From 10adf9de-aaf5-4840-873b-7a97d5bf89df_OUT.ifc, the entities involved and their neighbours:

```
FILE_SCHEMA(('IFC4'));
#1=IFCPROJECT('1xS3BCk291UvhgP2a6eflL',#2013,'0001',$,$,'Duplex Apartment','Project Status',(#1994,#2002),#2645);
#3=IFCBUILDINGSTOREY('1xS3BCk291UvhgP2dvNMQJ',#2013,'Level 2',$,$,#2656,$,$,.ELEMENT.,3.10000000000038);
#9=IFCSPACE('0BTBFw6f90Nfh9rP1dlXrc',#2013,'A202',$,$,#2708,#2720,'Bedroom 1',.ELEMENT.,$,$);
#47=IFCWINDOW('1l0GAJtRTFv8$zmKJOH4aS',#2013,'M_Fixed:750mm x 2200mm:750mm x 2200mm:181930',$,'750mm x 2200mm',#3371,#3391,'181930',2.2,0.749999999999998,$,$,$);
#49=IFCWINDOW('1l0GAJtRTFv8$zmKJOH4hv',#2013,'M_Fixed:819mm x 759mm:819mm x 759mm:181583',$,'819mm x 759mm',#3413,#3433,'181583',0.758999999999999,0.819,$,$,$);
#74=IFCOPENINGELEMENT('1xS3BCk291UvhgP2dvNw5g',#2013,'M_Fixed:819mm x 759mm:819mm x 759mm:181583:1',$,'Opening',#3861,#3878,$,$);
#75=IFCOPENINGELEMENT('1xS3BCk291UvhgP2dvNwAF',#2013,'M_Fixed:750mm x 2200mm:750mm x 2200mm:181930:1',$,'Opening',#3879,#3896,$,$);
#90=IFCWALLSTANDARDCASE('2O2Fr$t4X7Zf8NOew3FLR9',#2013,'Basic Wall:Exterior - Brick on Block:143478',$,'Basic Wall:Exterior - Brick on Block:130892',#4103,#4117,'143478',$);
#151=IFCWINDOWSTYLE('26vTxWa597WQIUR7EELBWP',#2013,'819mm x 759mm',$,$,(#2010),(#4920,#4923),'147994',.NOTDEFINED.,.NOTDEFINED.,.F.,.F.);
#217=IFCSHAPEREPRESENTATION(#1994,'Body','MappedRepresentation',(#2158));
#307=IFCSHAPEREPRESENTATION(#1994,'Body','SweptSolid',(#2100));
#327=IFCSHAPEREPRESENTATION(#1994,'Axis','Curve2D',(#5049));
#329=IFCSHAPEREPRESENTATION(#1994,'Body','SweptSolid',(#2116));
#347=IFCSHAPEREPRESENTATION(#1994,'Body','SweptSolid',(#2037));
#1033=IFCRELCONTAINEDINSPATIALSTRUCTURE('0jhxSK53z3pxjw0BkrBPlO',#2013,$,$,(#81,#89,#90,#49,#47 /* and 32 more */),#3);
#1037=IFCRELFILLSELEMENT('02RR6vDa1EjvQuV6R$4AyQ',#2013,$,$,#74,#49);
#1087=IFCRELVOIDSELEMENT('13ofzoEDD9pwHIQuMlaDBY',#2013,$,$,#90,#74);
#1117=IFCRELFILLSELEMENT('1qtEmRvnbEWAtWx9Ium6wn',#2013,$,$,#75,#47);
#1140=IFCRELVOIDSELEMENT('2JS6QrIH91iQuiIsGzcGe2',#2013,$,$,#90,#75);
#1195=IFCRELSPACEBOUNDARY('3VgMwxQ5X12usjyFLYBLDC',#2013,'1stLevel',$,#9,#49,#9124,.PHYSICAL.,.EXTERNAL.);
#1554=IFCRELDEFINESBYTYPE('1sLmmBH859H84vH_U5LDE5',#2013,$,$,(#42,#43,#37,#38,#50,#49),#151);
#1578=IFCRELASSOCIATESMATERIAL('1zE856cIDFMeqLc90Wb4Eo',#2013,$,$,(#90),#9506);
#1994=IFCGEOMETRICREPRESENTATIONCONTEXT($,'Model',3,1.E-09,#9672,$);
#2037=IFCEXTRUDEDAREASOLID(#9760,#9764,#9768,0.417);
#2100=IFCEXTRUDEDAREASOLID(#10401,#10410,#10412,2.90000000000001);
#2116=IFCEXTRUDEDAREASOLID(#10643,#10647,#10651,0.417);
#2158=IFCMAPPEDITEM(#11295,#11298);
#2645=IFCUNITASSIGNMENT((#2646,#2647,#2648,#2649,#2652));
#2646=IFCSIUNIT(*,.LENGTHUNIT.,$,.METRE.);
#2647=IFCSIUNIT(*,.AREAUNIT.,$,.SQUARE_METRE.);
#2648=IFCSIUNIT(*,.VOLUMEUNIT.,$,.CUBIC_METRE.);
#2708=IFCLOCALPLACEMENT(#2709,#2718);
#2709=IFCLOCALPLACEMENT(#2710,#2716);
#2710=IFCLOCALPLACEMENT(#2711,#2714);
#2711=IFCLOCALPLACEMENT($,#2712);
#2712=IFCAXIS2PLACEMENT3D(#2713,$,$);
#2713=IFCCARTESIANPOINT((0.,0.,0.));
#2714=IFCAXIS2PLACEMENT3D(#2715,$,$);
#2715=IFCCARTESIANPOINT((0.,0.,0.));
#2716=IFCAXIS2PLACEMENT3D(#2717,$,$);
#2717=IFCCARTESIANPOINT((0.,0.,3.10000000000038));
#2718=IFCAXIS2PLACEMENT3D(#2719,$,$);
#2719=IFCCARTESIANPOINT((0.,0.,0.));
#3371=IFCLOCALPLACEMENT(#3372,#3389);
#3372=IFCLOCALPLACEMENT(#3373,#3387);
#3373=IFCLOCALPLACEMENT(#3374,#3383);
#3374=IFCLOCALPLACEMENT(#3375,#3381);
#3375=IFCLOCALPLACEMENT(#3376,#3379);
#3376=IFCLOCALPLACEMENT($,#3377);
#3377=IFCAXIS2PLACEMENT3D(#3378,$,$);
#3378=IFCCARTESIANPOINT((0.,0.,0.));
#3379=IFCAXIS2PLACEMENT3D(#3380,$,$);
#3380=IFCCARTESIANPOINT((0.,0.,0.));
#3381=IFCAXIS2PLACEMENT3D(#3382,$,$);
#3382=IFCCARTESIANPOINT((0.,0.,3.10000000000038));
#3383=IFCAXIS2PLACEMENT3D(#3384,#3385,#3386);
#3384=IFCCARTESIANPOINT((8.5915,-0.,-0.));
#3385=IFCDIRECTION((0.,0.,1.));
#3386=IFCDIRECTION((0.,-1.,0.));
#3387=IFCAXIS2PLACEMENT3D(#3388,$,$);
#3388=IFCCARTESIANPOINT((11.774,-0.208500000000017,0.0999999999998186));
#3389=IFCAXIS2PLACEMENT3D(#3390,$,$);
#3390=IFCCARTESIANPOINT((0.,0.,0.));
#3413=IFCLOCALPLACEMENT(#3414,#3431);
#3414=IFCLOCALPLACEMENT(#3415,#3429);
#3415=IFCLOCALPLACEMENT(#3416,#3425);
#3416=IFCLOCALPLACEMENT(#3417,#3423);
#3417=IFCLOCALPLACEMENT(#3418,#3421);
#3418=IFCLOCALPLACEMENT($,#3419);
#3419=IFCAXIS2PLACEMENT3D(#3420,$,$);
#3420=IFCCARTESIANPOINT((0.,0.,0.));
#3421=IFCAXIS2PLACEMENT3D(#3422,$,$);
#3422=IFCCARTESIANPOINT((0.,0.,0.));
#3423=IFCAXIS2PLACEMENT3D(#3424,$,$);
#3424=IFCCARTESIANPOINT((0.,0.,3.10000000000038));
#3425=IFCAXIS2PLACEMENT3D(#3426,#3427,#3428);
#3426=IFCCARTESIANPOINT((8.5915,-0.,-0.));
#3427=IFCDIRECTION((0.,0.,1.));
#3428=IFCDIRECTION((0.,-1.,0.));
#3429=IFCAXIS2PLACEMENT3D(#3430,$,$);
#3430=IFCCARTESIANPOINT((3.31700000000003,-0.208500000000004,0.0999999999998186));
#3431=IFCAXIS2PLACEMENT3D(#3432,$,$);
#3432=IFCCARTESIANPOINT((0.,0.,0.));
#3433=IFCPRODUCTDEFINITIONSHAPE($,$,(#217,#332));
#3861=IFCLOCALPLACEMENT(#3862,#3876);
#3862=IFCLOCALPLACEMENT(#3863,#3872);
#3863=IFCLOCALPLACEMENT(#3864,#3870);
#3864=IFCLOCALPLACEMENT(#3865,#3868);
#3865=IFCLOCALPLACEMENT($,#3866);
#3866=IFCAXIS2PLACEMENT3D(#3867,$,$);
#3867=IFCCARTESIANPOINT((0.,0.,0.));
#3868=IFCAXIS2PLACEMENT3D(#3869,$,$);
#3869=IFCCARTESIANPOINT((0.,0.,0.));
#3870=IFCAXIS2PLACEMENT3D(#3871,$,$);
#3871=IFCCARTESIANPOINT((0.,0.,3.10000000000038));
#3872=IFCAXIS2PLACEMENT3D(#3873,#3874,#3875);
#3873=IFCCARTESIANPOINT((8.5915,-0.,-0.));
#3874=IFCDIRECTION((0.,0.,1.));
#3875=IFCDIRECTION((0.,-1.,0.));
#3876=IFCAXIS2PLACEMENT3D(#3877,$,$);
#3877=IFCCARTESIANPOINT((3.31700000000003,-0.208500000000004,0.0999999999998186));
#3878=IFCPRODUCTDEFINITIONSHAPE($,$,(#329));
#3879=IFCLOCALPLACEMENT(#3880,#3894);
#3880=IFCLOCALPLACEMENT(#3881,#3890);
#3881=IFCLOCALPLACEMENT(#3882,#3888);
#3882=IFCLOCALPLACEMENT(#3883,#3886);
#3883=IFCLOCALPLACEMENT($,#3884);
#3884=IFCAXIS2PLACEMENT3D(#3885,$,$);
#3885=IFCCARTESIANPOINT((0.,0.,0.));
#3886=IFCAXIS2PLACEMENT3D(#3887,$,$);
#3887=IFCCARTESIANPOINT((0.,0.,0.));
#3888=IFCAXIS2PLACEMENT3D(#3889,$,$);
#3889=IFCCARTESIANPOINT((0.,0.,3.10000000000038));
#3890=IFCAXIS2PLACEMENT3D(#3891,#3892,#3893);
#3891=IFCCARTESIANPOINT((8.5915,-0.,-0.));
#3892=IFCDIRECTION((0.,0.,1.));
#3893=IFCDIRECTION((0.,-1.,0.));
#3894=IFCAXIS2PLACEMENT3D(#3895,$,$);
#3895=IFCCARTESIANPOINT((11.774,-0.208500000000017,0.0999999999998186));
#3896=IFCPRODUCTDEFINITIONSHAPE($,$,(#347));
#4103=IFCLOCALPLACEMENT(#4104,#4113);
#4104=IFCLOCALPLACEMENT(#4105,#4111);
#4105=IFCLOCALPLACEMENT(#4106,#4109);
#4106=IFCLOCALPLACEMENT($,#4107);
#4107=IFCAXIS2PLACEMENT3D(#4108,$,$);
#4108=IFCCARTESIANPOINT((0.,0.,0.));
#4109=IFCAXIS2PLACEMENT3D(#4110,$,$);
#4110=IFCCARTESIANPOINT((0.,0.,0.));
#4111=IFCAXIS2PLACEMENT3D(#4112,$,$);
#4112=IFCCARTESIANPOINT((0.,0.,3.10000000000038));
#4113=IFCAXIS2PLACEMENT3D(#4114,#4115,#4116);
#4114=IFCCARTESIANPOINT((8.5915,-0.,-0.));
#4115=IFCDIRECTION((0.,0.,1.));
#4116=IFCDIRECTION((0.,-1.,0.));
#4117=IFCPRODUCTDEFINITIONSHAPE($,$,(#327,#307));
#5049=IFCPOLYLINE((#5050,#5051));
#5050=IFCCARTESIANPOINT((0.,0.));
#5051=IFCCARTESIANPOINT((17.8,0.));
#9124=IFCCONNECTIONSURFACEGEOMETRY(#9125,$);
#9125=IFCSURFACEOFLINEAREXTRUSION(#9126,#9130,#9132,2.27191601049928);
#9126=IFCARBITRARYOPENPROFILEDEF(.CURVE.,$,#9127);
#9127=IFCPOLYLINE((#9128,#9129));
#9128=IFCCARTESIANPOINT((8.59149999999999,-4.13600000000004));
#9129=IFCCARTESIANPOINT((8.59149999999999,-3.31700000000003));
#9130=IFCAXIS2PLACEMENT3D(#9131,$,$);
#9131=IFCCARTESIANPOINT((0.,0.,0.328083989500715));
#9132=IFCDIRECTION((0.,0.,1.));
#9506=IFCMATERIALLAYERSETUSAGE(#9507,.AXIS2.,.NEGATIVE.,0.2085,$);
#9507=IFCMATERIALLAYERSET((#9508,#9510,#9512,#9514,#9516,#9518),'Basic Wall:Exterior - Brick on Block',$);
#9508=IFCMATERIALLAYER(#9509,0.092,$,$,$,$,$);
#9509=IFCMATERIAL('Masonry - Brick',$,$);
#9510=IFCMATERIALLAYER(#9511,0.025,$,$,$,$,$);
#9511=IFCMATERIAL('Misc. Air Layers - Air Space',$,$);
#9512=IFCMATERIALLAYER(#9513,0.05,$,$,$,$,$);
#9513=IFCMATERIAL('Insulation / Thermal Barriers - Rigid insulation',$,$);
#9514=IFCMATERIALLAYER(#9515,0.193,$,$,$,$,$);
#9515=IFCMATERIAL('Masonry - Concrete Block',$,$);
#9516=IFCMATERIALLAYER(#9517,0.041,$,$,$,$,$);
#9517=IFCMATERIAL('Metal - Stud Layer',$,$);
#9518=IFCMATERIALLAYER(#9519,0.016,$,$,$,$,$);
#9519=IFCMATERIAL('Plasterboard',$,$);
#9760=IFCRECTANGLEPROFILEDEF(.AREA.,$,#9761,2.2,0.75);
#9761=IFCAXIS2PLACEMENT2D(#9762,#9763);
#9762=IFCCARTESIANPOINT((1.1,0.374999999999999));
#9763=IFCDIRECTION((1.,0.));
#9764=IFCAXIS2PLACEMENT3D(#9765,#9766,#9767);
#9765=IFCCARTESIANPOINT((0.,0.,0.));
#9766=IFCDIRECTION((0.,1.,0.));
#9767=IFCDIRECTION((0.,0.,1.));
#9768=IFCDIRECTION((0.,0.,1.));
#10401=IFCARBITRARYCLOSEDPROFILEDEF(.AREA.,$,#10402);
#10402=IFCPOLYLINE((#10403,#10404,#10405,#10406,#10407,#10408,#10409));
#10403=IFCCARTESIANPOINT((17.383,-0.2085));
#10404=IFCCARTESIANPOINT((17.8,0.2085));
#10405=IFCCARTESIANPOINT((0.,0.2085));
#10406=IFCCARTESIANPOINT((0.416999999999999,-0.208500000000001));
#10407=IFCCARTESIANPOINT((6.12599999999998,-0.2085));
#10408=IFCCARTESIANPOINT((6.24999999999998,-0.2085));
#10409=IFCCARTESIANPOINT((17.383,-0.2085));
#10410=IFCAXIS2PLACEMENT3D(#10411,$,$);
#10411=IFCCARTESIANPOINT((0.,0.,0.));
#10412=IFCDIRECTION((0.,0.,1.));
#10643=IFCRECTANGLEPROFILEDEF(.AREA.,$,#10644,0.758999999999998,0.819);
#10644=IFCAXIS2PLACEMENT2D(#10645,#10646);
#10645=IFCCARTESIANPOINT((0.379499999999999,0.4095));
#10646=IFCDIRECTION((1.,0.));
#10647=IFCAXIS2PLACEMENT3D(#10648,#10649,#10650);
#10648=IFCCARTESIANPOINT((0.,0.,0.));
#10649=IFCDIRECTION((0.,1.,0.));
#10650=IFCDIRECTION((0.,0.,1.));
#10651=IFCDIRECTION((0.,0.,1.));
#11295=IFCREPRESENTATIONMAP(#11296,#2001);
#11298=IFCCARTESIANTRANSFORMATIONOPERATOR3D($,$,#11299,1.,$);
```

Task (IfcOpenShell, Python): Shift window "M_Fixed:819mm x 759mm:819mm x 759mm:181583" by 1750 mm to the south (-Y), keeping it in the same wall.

```python
import numpy as np
import ifcopenshell
import ifcopenshell.api.geometry
import ifcopenshell.util.placement
import ifcopenshell.util.unit

model = ifcopenshell.open("10adf9de-aaf5-4840-873b-7a97d5bf89df_OUT.ifc")
unit_scale = ifcopenshell.util.unit.calculate_unit_scale(model)

window = model.by_guid("1l0GAJtRTFv8$zmKJOH4hv")
opening = window.FillsVoids[0].RelatingOpeningElement
wall = opening.VoidsElements[0].RelatingBuildingElement

wall_matrix = ifcopenshell.util.placement.get_local_placement(wall.ObjectPlacement)
shift = wall_matrix[:3, 0] * 1.75 / unit_scale
before = ifcopenshell.util.placement.get_local_placement(window.ObjectPlacement)[:3, 3].copy()

# The window is not placed relative to its opening, so move both.
for product in (opening, window):
    matrix = ifcopenshell.util.placement.get_local_placement(product.ObjectPlacement)
    matrix[:3, 3] += shift
    ifcopenshell.api.geometry.edit_object_placement(model, product=product, matrix=matrix, is_si=False)

# Space boundary surfaces are stored in each space's coordinates; move them too.
for rel in window.ProvidesBoundaries:
    if not rel.ConnectionGeometry:
        continue
    surface = rel.ConnectionGeometry.SurfaceOnRelatingElement
    space_matrix = ifcopenshell.util.placement.get_local_placement(rel.RelatingSpace.ObjectPlacement)
    point = np.array(surface.Position.Location.Coordinates) + space_matrix[:3, :3].T @ shift
    surface.Position = model.createIfcAxis2Placement3D(
        model.createIfcCartesianPoint(point.tolist()), surface.Position.Axis, surface.Position.RefDirection
    )

after = ifcopenshell.util.placement.get_local_placement(window.ObjectPlacement)[:3, 3]
print("window moved by", (after - before).round(3) + 0.0)

model.write("10adf9de-aaf5-4840-873b-7a97d5bf89df_OUT_v2.ifc")
```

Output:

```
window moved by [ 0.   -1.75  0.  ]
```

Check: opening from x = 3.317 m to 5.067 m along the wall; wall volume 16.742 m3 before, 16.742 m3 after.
